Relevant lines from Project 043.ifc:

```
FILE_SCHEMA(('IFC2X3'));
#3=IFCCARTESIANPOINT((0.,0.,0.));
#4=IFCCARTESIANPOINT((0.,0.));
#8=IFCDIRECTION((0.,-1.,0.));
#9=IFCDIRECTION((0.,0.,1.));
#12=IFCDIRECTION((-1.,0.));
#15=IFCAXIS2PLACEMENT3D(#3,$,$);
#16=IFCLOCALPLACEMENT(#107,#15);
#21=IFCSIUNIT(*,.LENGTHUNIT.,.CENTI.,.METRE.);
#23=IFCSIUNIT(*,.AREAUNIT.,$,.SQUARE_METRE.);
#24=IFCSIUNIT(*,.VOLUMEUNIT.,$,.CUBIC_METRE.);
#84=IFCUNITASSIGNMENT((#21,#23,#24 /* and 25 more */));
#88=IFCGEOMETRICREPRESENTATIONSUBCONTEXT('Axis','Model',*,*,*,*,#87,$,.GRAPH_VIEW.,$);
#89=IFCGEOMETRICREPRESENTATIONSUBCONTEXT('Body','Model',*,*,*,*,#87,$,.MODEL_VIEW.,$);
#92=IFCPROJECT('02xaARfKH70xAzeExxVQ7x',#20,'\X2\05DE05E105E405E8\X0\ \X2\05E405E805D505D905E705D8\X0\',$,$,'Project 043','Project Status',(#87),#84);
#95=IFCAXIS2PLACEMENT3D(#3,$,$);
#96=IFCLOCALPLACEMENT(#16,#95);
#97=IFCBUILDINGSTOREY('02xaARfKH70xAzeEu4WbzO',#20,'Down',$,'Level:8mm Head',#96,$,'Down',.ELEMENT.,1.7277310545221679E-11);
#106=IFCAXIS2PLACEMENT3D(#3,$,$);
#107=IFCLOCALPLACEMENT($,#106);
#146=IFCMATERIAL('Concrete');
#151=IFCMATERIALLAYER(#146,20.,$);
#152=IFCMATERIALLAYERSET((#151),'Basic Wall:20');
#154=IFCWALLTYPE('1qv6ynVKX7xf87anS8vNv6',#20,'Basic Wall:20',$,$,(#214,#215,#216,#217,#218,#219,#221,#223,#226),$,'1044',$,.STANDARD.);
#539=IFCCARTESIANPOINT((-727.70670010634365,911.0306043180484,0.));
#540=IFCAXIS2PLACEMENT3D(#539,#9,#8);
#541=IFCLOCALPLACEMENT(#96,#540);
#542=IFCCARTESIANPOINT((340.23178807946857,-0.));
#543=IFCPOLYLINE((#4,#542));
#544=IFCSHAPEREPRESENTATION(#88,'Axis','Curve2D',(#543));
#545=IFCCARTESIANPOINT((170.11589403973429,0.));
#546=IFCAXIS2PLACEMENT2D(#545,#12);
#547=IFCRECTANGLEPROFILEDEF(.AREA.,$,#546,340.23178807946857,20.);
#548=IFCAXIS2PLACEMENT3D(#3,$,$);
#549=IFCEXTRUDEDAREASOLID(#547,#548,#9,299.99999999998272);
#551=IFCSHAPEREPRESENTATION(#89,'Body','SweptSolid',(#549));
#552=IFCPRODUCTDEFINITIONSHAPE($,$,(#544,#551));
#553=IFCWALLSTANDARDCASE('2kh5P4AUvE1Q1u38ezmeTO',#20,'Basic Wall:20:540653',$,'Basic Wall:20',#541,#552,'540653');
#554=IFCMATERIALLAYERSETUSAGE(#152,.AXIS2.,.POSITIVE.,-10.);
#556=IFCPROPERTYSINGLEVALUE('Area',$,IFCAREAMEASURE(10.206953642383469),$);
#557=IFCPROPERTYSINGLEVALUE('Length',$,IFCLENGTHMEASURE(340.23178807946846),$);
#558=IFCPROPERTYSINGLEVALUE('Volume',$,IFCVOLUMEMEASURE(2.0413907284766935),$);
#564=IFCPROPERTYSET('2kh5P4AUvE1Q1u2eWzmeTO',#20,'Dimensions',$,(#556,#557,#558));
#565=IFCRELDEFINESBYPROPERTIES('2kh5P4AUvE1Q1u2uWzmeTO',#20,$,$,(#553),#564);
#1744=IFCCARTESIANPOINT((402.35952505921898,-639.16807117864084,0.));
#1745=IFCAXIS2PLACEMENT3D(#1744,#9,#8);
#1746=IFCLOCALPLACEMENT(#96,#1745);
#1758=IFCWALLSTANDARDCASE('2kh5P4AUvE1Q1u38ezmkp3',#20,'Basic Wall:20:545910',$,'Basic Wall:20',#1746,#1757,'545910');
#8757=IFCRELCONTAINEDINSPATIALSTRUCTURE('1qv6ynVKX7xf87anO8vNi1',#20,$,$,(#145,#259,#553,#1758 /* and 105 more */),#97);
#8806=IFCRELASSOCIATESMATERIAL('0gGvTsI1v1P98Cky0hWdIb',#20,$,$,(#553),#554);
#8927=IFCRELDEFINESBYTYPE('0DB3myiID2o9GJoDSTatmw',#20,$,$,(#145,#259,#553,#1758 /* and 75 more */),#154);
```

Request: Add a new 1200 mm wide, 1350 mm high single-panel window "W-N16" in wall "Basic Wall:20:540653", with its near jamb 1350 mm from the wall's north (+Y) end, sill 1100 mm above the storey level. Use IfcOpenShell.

```python
import numpy as np
import ifcopenshell
import ifcopenshell.api.feature
import ifcopenshell.api.geometry
import ifcopenshell.api.pset
import ifcopenshell.api.root
import ifcopenshell.api.spatial
import ifcopenshell.api.type
import ifcopenshell.geom
import ifcopenshell.util.element
import ifcopenshell.util.placement
import ifcopenshell.util.representation
import ifcopenshell.util.shape
import ifcopenshell.util.unit

model = ifcopenshell.open("Project 043.ifc")
unit_scale = ifcopenshell.util.unit.calculate_unit_scale(model)
area_scale = ifcopenshell.util.unit.calculate_unit_scale(model, "AREAUNIT")
volume_scale = ifcopenshell.util.unit.calculate_unit_scale(model, "VOLUMEUNIT")
settings = ifcopenshell.geom.settings()


def volume(element):
    """Net volume in cubic metres, openings subtracted."""
    shape = ifcopenshell.geom.create_shape(settings, element)
    return ifcopenshell.util.shape.get_volume(shape.geometry)


wall = model.by_id(553)
storey = ifcopenshell.util.element.get_container(wall, ifc_class="IfcBuildingStorey")
context = ifcopenshell.util.representation.get_context(model, "Model", "Body", "MODEL_VIEW")
before = volume(wall)

width, height, from_end, sill = 1.2, 1.35, 1.35, 1.1  # metres

# The wall runs along its own X axis, and the end named is its -X end.
wall_shape = ifcopenshell.geom.create_shape(settings, wall)
x, y, z = ifcopenshell.util.shape.get_vertices(wall_shape.geometry).T
start = x.min() + from_end
face, thickness = float(y.min()), float(y.max() - y.min())
wall_matrix = ifcopenshell.util.placement.get_local_placement(wall.ObjectPlacement)
level = ifcopenshell.util.placement.get_local_placement(storey.ObjectPlacement)[2, 3]


def in_wall(x, y):
    """Placement at x, y metres in the wall's axes, at sill height."""
    matrix = wall_matrix.copy()
    matrix[:, 3] = wall_matrix @ np.array([x / unit_scale, y / unit_scale, 0.0, 1.0])
    matrix[2, 3] = level + sill / unit_scale
    return matrix


# Opening: a box that overshoots both wall faces by 50 mm.
opening = ifcopenshell.api.root.create_entity(model, ifc_class="IfcOpeningElement")
box = ifcopenshell.api.geometry.add_wall_representation(
    model, context=context, length=width, height=height, thickness=thickness + 0.1
)
ifcopenshell.api.geometry.assign_representation(model, product=opening, representation=box)
ifcopenshell.api.geometry.edit_object_placement(model, product=opening, matrix=in_wall(start, face - 0.05), is_si=False)
ifcopenshell.api.feature.add_feature(model, feature=opening, element=wall)

window = ifcopenshell.api.root.create_entity(model, ifc_class="IfcWindow", name="W-N16")
window.OverallWidth, window.OverallHeight = width / unit_scale, height / unit_scale
body = ifcopenshell.api.geometry.add_window_representation(
    model,
    context=context,
    overall_width=window.OverallWidth,
    overall_height=window.OverallHeight,
    partition_type="SINGLE_PANEL",
)
ifcopenshell.api.geometry.assign_representation(model, product=window, representation=body)
ifcopenshell.api.spatial.assign_container(model, products=[window], relating_structure=storey)
fills = ifcopenshell.api.feature.add_filling(model, opening=opening, element=window)
fills.OwnerHistory = window.OwnerHistory  # required in IFC2X3

# IFC2X3 keeps the operation on the window style.
style = ifcopenshell.api.root.create_entity(model, ifc_class="IfcWindowStyle", name="W-N16")
style.OperationType, style.ConstructionType = "SINGLE_PANEL", "NOTDEFINED"
style.ParameterTakesPrecedence = style.Sizeable = False
ifcopenshell.api.type.assign_type(model, related_objects=[window], relating_type=style)

# Centre the window in the wall's thickness.
ifcopenshell.api.geometry.edit_object_placement(model, product=window, matrix=in_wall(start, face), is_si=False)
window_shape = ifcopenshell.geom.create_shape(settings, window)
depth = ifcopenshell.util.shape.get_vertices(window_shape.geometry)[:, 1]
offset = face + thickness / 2 - (depth.min() + depth.max()) / 2
ifcopenshell.api.geometry.edit_object_placement(model, product=window, matrix=in_wall(start, offset), is_si=False)

after = volume(wall)

# Update the wall's stored quantities.
pset = model.by_id(ifcopenshell.util.element.get_pset(wall, "Dimensions", should_inherit=False)["id"])
ifcopenshell.api.pset.edit_pset(model, pset=pset, properties={
    "Area": model.create_entity("IfcAreaMeasure", after / thickness / area_scale),
    "Volume": model.create_entity("IfcVolumeMeasure", after / volume_scale),
})

print(f"wall volume {before:.3f} -> {after:.3f} m3")

model.write("Project 043_v2.ifc")
```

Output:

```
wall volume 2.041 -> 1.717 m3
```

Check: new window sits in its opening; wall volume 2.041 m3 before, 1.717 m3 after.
